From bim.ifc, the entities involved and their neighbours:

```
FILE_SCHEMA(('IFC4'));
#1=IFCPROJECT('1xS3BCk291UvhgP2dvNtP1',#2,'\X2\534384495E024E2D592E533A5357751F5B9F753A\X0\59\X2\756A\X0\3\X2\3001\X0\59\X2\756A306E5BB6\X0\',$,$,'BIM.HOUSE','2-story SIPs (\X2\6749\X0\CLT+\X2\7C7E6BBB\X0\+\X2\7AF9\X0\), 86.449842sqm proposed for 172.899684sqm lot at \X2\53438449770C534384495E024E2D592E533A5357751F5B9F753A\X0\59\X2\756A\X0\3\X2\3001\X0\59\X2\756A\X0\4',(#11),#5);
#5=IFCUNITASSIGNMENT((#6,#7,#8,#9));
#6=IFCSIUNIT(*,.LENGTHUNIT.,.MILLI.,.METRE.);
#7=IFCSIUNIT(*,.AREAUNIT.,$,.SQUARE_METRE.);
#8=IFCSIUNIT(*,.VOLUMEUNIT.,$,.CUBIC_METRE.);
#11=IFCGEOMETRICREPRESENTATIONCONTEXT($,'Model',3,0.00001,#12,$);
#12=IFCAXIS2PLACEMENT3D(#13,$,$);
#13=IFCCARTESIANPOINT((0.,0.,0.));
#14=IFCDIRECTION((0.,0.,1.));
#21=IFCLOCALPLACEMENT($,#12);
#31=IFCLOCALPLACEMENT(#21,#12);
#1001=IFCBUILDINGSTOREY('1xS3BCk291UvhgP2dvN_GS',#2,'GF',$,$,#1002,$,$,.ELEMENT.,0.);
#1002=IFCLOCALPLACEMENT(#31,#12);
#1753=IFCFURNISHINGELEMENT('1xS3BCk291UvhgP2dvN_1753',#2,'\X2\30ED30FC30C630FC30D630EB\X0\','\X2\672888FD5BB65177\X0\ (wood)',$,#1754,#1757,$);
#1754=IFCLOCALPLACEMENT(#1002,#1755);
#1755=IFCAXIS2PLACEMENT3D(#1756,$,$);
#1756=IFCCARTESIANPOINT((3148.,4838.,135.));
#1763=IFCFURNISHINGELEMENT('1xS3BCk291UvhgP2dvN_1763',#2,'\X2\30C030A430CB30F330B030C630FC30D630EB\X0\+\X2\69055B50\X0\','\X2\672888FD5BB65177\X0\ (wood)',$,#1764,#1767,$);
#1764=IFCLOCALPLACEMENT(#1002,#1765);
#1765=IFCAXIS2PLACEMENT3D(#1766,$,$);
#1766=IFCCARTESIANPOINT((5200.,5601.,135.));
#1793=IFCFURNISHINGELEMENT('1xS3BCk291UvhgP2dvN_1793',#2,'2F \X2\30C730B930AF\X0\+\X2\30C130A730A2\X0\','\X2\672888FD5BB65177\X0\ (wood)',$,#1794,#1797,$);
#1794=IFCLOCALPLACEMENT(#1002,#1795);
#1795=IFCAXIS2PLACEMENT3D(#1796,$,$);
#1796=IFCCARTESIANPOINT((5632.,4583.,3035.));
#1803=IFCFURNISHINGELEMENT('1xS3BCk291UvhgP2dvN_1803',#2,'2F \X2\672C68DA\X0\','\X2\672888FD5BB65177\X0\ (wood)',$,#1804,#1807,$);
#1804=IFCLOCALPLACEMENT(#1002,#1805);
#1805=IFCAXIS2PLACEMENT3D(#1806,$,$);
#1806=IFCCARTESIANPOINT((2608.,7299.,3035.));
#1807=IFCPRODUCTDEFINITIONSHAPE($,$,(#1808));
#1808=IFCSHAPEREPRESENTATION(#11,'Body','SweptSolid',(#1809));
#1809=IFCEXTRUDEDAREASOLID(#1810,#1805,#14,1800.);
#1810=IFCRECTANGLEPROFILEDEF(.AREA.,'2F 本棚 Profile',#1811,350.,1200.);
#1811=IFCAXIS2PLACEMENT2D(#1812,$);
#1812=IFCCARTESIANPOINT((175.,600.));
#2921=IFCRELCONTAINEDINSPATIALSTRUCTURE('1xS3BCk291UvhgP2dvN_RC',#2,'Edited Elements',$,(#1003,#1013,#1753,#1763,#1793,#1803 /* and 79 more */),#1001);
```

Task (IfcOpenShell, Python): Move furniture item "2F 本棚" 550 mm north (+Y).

```python
import ifcopenshell
import ifcopenshell.api.geometry
import ifcopenshell.util.placement
import ifcopenshell.util.unit

model = ifcopenshell.open("bim.ifc")
unit_scale = ifcopenshell.util.unit.calculate_unit_scale(model)

item = model.by_id(1803)
matrix = ifcopenshell.util.placement.get_local_placement(item.ObjectPlacement)
matrix[1, 3] += 0.55 / unit_scale
ifcopenshell.api.geometry.edit_object_placement(model, product=item, matrix=matrix, is_si=False)

print(ifcopenshell.util.placement.get_local_placement(item.ObjectPlacement).round(3) + 0.0)

model.write("bim_edited.ifc")
```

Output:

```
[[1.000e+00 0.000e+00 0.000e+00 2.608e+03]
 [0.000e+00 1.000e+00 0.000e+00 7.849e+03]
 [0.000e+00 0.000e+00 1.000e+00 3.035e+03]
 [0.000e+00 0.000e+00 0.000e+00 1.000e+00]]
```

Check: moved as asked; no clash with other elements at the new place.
